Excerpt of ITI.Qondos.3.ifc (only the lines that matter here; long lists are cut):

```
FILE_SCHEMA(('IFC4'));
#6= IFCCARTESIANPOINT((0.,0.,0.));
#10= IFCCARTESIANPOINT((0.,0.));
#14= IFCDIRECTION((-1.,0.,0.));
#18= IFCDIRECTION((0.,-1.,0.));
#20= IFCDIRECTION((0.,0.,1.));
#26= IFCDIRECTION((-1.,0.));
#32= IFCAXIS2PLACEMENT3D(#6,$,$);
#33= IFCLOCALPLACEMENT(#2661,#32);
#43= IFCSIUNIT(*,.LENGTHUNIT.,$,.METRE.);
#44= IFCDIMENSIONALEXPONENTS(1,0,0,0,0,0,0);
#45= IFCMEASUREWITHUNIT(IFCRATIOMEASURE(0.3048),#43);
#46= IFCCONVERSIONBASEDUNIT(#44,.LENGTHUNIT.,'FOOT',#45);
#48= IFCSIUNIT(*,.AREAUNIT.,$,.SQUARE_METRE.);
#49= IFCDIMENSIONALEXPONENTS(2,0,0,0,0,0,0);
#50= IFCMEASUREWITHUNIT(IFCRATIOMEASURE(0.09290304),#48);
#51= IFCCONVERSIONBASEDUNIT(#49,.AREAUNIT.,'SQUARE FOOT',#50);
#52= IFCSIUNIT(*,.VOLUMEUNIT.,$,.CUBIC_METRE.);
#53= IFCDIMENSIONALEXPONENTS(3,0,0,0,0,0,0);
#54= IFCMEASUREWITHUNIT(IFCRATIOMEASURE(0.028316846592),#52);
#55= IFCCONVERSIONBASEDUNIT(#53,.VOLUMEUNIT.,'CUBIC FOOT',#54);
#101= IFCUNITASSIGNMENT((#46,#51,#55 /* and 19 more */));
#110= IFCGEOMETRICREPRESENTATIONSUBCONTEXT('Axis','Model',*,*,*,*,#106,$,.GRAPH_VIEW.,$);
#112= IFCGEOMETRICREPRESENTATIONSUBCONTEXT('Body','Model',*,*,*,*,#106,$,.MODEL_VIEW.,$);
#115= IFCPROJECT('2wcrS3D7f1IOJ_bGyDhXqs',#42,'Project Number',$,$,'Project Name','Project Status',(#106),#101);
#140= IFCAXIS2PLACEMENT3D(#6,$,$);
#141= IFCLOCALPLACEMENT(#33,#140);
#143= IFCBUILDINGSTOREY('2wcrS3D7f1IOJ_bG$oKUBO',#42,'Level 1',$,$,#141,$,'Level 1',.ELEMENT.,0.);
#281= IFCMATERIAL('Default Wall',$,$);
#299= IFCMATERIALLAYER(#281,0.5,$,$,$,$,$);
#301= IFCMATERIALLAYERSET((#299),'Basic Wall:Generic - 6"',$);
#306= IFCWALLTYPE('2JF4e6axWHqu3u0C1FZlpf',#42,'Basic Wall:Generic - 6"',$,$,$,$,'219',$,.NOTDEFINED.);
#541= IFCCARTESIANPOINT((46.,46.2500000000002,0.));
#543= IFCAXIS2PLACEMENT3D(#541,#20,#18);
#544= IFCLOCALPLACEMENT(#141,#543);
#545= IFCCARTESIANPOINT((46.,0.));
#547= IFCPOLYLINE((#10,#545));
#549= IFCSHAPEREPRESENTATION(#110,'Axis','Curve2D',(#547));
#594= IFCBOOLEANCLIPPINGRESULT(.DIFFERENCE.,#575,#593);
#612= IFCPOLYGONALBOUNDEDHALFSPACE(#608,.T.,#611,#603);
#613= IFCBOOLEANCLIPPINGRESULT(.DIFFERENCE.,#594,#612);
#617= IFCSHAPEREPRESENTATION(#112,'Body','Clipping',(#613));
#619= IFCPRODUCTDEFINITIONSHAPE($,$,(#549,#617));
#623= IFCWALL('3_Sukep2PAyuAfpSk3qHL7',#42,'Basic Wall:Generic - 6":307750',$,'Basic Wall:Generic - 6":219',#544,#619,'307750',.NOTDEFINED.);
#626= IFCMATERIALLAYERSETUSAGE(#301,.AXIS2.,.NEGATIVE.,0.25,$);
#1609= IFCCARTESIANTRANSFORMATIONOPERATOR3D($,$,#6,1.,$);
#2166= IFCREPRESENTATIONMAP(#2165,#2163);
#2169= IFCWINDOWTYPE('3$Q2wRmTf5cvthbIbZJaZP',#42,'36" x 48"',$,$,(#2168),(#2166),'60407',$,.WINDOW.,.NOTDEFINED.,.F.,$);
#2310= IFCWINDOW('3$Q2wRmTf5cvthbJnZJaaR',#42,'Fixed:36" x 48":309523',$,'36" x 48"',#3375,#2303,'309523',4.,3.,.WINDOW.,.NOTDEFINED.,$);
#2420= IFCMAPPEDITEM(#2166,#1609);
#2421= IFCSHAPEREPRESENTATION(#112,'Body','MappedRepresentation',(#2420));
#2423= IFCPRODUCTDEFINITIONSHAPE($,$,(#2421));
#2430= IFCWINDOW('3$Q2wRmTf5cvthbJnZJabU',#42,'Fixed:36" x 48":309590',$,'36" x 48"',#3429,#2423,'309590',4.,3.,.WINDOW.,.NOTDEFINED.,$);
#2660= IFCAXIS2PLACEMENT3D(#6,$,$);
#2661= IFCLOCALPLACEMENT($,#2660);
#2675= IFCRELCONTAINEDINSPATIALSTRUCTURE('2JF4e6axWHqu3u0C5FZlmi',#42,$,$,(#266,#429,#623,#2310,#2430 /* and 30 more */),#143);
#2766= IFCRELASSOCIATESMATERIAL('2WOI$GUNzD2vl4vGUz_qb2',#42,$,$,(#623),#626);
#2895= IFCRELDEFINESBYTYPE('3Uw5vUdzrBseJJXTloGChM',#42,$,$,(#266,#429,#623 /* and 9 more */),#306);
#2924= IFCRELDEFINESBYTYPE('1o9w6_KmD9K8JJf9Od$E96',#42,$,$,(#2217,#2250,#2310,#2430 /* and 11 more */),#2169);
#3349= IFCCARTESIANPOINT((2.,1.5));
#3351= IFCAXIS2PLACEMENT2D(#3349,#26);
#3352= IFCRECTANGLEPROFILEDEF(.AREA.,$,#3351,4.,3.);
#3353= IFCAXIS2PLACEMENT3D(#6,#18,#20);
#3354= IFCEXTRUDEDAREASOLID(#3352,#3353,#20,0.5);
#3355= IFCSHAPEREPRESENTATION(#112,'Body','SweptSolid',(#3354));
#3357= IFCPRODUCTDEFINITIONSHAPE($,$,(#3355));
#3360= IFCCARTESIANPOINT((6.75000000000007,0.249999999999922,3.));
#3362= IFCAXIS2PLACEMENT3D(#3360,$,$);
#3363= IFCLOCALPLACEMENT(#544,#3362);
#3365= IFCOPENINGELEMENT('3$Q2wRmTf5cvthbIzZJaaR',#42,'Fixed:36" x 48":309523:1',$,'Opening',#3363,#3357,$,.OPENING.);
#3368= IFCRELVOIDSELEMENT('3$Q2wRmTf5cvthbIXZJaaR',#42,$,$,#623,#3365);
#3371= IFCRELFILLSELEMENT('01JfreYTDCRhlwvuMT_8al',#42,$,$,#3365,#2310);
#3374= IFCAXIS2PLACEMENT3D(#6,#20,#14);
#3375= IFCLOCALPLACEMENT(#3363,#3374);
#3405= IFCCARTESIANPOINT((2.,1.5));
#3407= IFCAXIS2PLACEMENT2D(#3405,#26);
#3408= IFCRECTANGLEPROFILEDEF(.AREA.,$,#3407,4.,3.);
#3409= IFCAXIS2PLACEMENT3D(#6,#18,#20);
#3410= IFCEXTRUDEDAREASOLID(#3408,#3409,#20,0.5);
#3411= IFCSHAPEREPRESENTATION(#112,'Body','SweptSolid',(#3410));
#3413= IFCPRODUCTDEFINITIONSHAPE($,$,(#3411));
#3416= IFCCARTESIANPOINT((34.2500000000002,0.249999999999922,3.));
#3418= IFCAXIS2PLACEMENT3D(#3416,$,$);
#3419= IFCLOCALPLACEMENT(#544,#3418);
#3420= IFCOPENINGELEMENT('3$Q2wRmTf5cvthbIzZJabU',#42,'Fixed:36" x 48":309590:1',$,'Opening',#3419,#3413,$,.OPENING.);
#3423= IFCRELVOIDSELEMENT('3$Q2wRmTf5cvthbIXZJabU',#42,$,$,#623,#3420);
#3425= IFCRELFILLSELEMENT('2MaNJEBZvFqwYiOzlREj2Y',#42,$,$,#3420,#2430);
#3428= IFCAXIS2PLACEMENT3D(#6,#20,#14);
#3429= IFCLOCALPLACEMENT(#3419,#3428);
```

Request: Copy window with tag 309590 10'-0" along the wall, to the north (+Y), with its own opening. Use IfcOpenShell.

```python
import ifcopenshell
import ifcopenshell.api.feature
import ifcopenshell.api.geometry
import ifcopenshell.api.root
import ifcopenshell.geom
import ifcopenshell.util.element
import ifcopenshell.util.placement
import ifcopenshell.util.shape
import ifcopenshell.util.unit

model = ifcopenshell.open("ITI.Qondos.3.ifc")
unit_scale = ifcopenshell.util.unit.calculate_unit_scale(model)
settings = ifcopenshell.geom.settings()


def volume(element):
    """Net volume in cubic metres, openings subtracted."""
    shape = ifcopenshell.geom.create_shape(settings, element)
    return ifcopenshell.util.shape.get_volume(shape.geometry)


def reuse_history(source, copy):
    """copy_class also copies each property set's owner history, people and application; keep the originals."""
    for rel in copy.IsDefinedBy:
        if rel.is_a("IfcRelDefinesByProperties") and (history := rel.RelatingPropertyDefinition.OwnerHistory):
            rel.RelatingPropertyDefinition.OwnerHistory = source.OwnerHistory
            ifcopenshell.util.element.remove_deep2(model, history)


window = model.by_guid("3$Q2wRmTf5cvthbJnZJabU")
opening = window.FillsVoids[0].RelatingOpeningElement
wall = opening.VoidsElements[0].RelatingBuildingElement
before = volume(wall)
shift = ifcopenshell.util.placement.get_local_placement(wall.ObjectPlacement)[:3, 0] * -120 * 0.0254 / unit_scale

# copy_class copies the void relationship, type, container and properties, but no geometry.
new_opening = ifcopenshell.api.root.copy_class(model, product=opening)
new_opening.Representation = ifcopenshell.util.element.copy_deep(
    model, opening.Representation, exclude=["IfcGeometricRepresentationContext", "IfcRepresentationMap"]
)
new_opening.Name = 'Fixed:36" x 48"'
new_window = ifcopenshell.api.root.copy_class(model, product=window)
new_window.Representation = ifcopenshell.util.element.copy_deep(
    model, window.Representation, exclude=["IfcGeometricRepresentationContext", "IfcRepresentationMap"]
)
new_window.Name = 'Fixed:36" x 48"'
new_window.Tag = None
reuse_history(window, new_window)
ifcopenshell.api.feature.add_filling(model, opening=new_opening, element=new_window)

for old, new in ((opening, new_opening), (window, new_window)):
    matrix = ifcopenshell.util.placement.get_local_placement(old.ObjectPlacement)
    matrix[:3, 3] += shift
    ifcopenshell.api.geometry.edit_object_placement(model, product=new, matrix=matrix, is_si=False)

after = volume(wall)

print(f"wall volume {before:.3f} -> {after:.3f} m3")

model.write("ITI.Qondos.3_rev.ifc")
```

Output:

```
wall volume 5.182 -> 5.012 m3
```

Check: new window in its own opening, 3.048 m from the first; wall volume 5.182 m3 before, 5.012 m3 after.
